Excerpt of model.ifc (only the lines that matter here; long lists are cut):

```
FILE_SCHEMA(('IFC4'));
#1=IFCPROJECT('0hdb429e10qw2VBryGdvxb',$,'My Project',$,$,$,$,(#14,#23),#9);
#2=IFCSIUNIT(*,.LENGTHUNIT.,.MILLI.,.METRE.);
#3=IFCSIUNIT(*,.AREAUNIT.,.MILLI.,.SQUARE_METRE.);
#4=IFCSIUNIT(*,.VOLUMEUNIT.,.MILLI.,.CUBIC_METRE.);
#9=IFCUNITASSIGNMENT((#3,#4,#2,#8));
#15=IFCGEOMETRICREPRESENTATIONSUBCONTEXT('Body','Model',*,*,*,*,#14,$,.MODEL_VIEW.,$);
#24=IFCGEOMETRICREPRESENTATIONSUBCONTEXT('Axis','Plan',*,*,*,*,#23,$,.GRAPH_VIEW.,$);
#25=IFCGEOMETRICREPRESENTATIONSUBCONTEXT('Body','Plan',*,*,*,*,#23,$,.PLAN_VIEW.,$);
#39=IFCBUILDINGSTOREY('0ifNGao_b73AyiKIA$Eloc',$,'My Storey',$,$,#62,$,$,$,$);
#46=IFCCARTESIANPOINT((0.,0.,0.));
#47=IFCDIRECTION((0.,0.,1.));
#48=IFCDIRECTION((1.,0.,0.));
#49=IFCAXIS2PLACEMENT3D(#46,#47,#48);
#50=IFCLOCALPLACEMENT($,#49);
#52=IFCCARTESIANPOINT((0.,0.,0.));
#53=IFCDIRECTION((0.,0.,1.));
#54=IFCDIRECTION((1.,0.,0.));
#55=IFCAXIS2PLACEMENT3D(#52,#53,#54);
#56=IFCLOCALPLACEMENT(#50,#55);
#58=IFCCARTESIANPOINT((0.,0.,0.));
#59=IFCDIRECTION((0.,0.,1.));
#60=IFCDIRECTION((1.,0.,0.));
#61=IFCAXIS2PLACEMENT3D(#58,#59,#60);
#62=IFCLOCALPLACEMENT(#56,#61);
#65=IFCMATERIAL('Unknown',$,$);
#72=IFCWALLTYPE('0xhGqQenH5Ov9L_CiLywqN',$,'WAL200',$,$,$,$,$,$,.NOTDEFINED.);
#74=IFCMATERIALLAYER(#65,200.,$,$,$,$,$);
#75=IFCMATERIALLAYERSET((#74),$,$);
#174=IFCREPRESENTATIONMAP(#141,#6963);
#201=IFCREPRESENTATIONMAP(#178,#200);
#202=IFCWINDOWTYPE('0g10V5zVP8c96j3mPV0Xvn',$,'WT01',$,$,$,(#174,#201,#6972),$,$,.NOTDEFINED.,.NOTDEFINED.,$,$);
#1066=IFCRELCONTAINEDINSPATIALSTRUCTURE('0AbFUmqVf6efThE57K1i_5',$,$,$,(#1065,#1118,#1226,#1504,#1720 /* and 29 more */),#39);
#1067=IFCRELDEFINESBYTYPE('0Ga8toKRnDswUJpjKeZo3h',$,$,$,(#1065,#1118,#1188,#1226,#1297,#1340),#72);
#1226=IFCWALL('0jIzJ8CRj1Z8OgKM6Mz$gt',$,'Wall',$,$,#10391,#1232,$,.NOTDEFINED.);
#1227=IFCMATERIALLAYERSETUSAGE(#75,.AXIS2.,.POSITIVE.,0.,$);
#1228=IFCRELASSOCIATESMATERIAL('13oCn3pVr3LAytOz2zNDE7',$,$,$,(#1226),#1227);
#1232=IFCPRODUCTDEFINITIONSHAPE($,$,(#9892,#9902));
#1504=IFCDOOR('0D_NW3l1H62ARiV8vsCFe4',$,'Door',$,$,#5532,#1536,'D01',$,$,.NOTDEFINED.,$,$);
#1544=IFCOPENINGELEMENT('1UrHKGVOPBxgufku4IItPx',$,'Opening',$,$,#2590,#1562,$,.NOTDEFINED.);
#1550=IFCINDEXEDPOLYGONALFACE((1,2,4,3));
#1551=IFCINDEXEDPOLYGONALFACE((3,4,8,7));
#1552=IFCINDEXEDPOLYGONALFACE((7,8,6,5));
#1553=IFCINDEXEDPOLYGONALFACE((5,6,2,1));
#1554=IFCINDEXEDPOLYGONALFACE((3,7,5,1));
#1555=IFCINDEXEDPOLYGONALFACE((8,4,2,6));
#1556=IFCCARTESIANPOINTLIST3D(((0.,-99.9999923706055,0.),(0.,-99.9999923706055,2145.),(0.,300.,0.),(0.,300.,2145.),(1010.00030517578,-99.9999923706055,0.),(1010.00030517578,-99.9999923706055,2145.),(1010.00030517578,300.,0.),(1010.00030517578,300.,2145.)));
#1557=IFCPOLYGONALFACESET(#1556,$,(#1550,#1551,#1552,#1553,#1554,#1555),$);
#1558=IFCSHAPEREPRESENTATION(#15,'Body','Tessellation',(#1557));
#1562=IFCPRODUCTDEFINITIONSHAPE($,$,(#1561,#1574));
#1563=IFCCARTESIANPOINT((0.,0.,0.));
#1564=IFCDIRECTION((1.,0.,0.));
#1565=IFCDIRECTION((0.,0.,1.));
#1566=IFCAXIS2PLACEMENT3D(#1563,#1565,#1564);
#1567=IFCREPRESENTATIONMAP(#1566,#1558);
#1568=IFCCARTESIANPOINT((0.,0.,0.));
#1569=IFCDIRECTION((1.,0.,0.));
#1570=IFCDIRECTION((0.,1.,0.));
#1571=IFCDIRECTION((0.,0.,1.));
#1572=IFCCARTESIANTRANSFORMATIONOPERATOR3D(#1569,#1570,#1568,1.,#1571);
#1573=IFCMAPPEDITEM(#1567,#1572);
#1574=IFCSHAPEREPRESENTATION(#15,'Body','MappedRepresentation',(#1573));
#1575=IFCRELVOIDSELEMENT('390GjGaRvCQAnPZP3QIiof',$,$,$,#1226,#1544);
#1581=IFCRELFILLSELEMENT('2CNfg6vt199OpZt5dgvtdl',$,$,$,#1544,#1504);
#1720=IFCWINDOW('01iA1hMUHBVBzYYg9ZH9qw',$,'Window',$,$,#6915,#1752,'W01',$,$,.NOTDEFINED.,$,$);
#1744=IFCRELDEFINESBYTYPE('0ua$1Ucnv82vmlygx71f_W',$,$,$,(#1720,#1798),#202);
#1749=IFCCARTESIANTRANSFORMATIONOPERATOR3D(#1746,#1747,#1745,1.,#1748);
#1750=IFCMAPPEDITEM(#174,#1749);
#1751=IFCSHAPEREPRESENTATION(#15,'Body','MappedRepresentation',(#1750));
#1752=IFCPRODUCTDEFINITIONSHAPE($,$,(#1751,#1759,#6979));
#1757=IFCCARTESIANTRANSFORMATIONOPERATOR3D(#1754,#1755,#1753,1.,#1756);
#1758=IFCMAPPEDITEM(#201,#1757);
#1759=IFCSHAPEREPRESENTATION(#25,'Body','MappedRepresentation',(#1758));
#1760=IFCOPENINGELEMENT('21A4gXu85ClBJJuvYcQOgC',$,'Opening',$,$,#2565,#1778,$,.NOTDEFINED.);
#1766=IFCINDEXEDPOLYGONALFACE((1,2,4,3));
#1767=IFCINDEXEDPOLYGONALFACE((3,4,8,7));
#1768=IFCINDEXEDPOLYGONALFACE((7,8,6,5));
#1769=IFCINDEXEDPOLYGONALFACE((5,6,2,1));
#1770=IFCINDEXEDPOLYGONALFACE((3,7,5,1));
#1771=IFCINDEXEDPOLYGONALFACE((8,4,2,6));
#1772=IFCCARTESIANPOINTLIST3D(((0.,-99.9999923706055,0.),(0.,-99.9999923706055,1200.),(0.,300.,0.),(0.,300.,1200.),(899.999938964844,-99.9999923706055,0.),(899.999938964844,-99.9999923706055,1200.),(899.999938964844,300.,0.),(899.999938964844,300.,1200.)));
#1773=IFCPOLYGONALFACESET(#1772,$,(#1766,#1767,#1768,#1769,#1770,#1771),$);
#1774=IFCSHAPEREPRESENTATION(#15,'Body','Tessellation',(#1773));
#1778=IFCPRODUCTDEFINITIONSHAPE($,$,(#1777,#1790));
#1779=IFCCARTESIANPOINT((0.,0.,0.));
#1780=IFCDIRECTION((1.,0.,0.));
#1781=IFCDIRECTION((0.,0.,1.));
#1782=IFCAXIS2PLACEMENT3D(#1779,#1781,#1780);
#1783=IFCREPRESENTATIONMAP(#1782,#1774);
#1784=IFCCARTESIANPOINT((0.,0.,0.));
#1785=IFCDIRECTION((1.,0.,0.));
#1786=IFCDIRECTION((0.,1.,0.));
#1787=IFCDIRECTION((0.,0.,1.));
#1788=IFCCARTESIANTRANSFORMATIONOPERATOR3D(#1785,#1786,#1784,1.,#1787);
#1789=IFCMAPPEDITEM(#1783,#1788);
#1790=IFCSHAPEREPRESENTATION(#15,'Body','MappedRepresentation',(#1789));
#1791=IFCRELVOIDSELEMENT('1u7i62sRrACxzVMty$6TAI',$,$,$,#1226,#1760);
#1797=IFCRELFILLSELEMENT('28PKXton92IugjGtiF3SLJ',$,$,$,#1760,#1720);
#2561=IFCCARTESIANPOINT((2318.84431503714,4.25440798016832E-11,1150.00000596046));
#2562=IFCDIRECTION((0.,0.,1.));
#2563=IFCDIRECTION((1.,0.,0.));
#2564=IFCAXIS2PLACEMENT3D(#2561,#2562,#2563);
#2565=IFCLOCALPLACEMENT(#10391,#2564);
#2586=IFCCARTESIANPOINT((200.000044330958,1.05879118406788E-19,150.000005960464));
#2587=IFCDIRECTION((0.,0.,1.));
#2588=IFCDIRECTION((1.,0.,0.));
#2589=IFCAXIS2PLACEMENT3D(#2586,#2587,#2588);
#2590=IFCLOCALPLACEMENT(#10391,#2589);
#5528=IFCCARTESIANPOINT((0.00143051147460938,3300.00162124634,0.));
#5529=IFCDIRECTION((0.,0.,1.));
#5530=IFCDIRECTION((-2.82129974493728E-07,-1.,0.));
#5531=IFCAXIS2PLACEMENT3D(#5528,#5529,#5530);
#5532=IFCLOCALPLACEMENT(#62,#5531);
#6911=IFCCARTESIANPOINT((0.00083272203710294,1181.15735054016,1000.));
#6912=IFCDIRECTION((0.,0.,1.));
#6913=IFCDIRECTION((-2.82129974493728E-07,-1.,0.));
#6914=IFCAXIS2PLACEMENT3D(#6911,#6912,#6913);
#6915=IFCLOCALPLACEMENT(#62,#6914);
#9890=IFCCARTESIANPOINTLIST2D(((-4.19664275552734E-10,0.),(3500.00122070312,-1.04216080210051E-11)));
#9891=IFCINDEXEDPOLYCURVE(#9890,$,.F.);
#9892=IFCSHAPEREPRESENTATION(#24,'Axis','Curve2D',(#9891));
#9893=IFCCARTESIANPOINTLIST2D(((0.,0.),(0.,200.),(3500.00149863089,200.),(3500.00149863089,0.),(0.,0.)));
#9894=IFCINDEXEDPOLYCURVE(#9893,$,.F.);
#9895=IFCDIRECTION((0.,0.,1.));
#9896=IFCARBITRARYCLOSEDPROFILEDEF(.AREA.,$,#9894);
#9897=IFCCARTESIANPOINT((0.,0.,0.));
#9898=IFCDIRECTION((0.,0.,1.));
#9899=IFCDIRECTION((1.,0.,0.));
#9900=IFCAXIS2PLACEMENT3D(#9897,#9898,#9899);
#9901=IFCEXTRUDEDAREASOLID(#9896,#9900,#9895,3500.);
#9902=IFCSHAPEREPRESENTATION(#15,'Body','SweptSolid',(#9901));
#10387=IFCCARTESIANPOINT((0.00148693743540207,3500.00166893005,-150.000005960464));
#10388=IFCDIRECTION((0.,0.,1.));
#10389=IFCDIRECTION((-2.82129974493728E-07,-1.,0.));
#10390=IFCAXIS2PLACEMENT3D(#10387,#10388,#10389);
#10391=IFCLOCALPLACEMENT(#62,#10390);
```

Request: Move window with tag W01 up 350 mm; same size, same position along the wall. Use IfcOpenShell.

```python
import numpy as np
import ifcopenshell
import ifcopenshell.api.geometry
import ifcopenshell.util.placement
import ifcopenshell.util.unit

model = ifcopenshell.open("model.ifc")
unit_scale = ifcopenshell.util.unit.calculate_unit_scale(model)

window = model.by_guid("01iA1hMUHBVBzYYg9ZH9qw")
opening = window.FillsVoids[0].RelatingOpeningElement
dz = 0.35 / unit_scale

shift = np.array([0.0, 0.0, dz])
# The window is not placed relative to its opening, so move both.
for product in (opening, window):
    matrix = ifcopenshell.util.placement.get_local_placement(product.ObjectPlacement)
    matrix[:3, 3] += shift
    ifcopenshell.api.geometry.edit_object_placement(model, product=product, matrix=matrix, is_si=False)

print(f"moved by {dz * unit_scale:+.3f} m")

model.write("model_updated.ifc")
```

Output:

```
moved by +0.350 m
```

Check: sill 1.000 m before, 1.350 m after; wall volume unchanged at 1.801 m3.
